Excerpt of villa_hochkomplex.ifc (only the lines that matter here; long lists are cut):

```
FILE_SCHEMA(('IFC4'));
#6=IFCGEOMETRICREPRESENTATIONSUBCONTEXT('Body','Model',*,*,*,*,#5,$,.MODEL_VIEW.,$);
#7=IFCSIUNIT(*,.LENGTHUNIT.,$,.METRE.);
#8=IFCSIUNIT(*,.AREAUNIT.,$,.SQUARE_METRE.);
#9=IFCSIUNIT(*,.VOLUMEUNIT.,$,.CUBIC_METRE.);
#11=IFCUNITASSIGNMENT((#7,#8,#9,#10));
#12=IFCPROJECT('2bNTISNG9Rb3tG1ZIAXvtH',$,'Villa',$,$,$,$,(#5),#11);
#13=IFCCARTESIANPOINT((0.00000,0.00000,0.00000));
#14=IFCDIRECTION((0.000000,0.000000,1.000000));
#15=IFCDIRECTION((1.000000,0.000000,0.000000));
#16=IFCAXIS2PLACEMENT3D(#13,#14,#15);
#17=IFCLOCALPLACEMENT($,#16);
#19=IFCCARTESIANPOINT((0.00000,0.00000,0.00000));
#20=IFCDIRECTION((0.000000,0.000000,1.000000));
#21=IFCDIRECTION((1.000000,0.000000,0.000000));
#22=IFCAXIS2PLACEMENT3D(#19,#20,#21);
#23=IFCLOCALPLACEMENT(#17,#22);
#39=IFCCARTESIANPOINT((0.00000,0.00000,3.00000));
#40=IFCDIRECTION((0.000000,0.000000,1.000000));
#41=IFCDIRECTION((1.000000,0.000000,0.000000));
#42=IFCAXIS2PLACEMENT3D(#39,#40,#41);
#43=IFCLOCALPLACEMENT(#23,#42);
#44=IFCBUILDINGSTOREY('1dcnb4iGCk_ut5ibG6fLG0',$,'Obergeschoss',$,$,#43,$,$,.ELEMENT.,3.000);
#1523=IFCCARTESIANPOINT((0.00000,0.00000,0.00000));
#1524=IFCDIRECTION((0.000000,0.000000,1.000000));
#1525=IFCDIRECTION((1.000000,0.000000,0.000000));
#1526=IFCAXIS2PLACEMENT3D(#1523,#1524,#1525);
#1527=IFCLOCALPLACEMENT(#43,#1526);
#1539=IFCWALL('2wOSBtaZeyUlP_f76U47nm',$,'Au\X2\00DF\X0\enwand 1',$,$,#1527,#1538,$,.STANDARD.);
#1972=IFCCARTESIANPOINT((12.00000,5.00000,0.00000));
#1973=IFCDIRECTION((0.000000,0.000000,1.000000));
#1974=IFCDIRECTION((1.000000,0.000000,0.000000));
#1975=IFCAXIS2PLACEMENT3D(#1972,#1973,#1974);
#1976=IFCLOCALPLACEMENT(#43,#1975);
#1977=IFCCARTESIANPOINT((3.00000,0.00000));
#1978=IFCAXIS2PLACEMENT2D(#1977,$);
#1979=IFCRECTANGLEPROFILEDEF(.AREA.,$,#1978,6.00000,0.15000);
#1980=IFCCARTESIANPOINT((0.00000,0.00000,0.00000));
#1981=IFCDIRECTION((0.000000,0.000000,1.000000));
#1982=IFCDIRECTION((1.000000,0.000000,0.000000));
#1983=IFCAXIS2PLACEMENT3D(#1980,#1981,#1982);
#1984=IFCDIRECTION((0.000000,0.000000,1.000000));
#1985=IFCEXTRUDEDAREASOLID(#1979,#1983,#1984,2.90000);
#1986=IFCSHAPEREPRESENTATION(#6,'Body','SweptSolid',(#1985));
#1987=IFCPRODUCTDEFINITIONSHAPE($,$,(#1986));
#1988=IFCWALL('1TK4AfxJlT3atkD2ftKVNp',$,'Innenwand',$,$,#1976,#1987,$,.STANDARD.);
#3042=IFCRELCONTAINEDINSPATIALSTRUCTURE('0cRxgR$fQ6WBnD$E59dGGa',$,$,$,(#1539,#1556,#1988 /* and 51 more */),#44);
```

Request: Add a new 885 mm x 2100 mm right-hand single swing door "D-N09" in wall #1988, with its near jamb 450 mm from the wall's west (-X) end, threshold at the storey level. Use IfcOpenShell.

```python
import numpy as np
import ifcopenshell
import ifcopenshell.api.feature
import ifcopenshell.api.geometry
import ifcopenshell.api.root
import ifcopenshell.api.spatial
import ifcopenshell.geom
import ifcopenshell.util.element
import ifcopenshell.util.placement
import ifcopenshell.util.representation
import ifcopenshell.util.shape
import ifcopenshell.util.unit

model = ifcopenshell.open("villa_hochkomplex.ifc")
unit_scale = ifcopenshell.util.unit.calculate_unit_scale(model)
settings = ifcopenshell.geom.settings()


def volume(element):
    """Net volume in cubic metres, openings subtracted."""
    shape = ifcopenshell.geom.create_shape(settings, element)
    return ifcopenshell.util.shape.get_volume(shape.geometry)


wall = model.by_guid("1TK4AfxJlT3atkD2ftKVNp")
storey = ifcopenshell.util.element.get_container(wall, ifc_class="IfcBuildingStorey")
context = ifcopenshell.util.representation.get_context(model, "Model", "Body", "MODEL_VIEW")
before = volume(wall)

width, height, from_end, sill = 0.885, 2.1, 0.45, 0.0  # metres

# The wall runs along its own X axis, and the end named is its -X end.
wall_shape = ifcopenshell.geom.create_shape(settings, wall)
x, y, z = ifcopenshell.util.shape.get_vertices(wall_shape.geometry).T
start = x.min() + from_end
face, thickness = float(y.min()), float(y.max() - y.min())
wall_matrix = ifcopenshell.util.placement.get_local_placement(wall.ObjectPlacement)
level = ifcopenshell.util.placement.get_local_placement(storey.ObjectPlacement)[2, 3]


def in_wall(x, y):
    """Placement at x, y metres in the wall's axes, at sill height."""
    matrix = wall_matrix.copy()
    matrix[:, 3] = wall_matrix @ np.array([x / unit_scale, y / unit_scale, 0.0, 1.0])
    matrix[2, 3] = level + sill / unit_scale
    return matrix


# Opening: a box that overshoots both wall faces by 50 mm.
opening = ifcopenshell.api.root.create_entity(model, ifc_class="IfcOpeningElement", predefined_type="OPENING")
box = ifcopenshell.api.geometry.add_wall_representation(
    model, context=context, length=width, height=height, thickness=thickness + 0.1
)
ifcopenshell.api.geometry.assign_representation(model, product=opening, representation=box)
ifcopenshell.api.geometry.edit_object_placement(model, product=opening, matrix=in_wall(start, face - 0.05), is_si=False)
ifcopenshell.api.feature.add_feature(model, feature=opening, element=wall)

door = ifcopenshell.api.root.create_entity(model, ifc_class="IfcDoor", name="D-N09", predefined_type="DOOR")
door.OverallWidth, door.OverallHeight = width / unit_scale, height / unit_scale
door.OperationType = "SINGLE_SWING_RIGHT"
body = ifcopenshell.api.geometry.add_door_representation(
    model,
    context=context,
    overall_width=door.OverallWidth,
    overall_height=door.OverallHeight,
    operation_type="SINGLE_SWING_RIGHT",
    lining_properties={"LiningDepth": thickness / unit_scale, "ThresholdDepth": thickness / unit_scale},
)
ifcopenshell.api.geometry.assign_representation(model, product=door, representation=body)
ifcopenshell.api.spatial.assign_container(model, products=[door], relating_structure=storey)
ifcopenshell.api.feature.add_filling(model, opening=opening, element=door)

# The lining spans the wall, so the door starts at the wall face.
ifcopenshell.api.geometry.edit_object_placement(model, product=door, matrix=in_wall(start, face), is_si=False)

after = volume(wall)

print(f"wall volume {before:.3f} -> {after:.3f} m3")

model.write("villa_hochkomplex_edited.ifc")
```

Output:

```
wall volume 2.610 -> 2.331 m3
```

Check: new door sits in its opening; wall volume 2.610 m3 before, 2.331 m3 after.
